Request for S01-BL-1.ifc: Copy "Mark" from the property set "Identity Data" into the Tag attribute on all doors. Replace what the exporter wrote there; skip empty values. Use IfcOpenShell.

First a look at what the model holds.

```python
import ifcopenshell
import ifcopenshell.util.element

model = ifcopenshell.open("S01-BL-1.ifc")
print(model.schema)
doors = model.by_type("IfcDoor")
print(len(doors), "doors")
for e in doors[:8]:
    source = ifcopenshell.util.element.get_pset(e, "Identity Data", "Mark")
    target = e.Tag
    print(e.id(), repr(source), repr(target), sep=" | ")
```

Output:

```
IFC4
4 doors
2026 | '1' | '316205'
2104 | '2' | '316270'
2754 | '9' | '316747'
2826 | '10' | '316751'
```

```python
import ifcopenshell
import ifcopenshell.util.element

model = ifcopenshell.open("S01-BL-1.ifc")

count = 0
for e in model.by_type("IfcDoor"):
    value = ifcopenshell.util.element.get_pset(e, "Identity Data", "Mark")
    current = e.Tag
    if not value or not value.strip() or current == value:
        continue
    e.Tag = value
    count += 1

print(count, "doors updated")

model.write("S01-BL-1_v2.ifc")
```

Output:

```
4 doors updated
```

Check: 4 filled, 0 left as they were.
